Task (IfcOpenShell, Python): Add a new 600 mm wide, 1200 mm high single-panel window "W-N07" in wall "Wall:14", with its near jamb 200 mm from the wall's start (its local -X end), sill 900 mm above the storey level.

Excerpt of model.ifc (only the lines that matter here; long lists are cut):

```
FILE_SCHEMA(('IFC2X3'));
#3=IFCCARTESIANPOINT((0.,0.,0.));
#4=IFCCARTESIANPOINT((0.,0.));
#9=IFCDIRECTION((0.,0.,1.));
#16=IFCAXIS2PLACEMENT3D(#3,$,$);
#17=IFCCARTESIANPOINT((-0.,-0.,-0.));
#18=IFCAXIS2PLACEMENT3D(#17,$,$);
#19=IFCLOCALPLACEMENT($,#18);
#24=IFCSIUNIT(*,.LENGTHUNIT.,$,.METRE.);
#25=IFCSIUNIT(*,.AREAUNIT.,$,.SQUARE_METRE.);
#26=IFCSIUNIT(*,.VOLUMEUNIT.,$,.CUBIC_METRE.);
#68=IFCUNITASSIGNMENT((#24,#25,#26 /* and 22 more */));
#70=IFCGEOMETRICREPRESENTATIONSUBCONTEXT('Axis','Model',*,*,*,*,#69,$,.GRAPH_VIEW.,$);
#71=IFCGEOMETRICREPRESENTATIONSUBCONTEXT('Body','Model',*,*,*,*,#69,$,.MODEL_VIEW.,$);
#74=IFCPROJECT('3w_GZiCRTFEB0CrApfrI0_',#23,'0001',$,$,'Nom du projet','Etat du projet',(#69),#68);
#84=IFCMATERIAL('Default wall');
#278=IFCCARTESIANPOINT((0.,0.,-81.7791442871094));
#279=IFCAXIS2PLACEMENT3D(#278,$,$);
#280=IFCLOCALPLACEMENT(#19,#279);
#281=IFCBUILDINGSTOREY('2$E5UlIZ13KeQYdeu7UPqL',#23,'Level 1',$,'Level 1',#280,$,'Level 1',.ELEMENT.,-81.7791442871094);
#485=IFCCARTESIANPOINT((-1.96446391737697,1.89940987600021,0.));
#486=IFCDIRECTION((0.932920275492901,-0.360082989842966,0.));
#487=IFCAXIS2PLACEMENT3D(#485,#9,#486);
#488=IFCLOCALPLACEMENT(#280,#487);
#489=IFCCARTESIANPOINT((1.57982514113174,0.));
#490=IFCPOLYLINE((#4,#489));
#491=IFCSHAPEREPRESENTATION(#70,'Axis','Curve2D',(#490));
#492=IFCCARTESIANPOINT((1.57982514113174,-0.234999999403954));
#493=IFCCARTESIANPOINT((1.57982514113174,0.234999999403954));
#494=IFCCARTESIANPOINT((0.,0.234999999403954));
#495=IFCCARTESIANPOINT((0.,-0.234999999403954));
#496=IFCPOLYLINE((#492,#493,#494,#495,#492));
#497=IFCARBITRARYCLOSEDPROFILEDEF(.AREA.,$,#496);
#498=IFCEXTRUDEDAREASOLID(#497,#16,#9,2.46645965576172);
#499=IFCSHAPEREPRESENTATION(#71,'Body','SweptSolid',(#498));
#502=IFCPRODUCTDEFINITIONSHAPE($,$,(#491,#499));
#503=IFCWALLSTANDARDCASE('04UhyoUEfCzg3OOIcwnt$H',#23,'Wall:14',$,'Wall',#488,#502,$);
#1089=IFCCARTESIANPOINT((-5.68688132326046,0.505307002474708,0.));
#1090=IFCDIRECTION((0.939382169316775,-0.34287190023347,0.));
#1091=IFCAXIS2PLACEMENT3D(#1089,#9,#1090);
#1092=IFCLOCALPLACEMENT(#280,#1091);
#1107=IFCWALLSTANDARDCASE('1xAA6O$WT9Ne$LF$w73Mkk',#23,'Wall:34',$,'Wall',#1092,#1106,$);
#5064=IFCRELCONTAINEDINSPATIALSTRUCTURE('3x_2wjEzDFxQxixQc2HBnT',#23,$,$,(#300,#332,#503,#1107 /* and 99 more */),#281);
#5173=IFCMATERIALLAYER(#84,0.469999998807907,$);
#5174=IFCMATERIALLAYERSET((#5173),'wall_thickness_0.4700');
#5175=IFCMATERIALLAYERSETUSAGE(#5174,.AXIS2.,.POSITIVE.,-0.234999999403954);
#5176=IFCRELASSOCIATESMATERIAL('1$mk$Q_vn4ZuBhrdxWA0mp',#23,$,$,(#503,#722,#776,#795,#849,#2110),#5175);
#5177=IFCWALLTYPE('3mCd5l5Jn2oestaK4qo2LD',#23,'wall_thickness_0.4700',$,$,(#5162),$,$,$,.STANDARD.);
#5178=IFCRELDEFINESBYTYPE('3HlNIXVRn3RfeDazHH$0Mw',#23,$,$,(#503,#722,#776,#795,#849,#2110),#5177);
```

```python
import numpy as np
import ifcopenshell
import ifcopenshell.api.feature
import ifcopenshell.api.geometry
import ifcopenshell.api.root
import ifcopenshell.api.spatial
import ifcopenshell.api.type
import ifcopenshell.geom
import ifcopenshell.util.element
import ifcopenshell.util.placement
import ifcopenshell.util.representation
import ifcopenshell.util.shape
import ifcopenshell.util.unit

model = ifcopenshell.open("model.ifc")
unit_scale = ifcopenshell.util.unit.calculate_unit_scale(model)
settings = ifcopenshell.geom.settings()


def volume(element):
    """Net volume in cubic metres, openings subtracted."""
    shape = ifcopenshell.geom.create_shape(settings, element)
    return ifcopenshell.util.shape.get_volume(shape.geometry)


wall = model.by_id(503)
storey = ifcopenshell.util.element.get_container(wall, ifc_class="IfcBuildingStorey")
context = ifcopenshell.util.representation.get_context(model, "Model", "Body", "MODEL_VIEW")
before = volume(wall)

width, height, from_end, sill = 0.6, 1.2, 0.2, 0.9  # metres

# The wall runs along its own X axis, and the end named is its -X end.
wall_shape = ifcopenshell.geom.create_shape(settings, wall)
x, y, z = ifcopenshell.util.shape.get_vertices(wall_shape.geometry).T
start = x.min() + from_end
face, thickness = float(y.min()), float(y.max() - y.min())
wall_matrix = ifcopenshell.util.placement.get_local_placement(wall.ObjectPlacement)
level = ifcopenshell.util.placement.get_local_placement(storey.ObjectPlacement)[2, 3]


def in_wall(x, y):
    """Placement at x, y metres in the wall's axes, at sill height."""
    matrix = wall_matrix.copy()
    matrix[:, 3] = wall_matrix @ np.array([x / unit_scale, y / unit_scale, 0.0, 1.0])
    matrix[2, 3] = level + sill / unit_scale
    return matrix


# Opening: a box that overshoots both wall faces by 50 mm.
opening = ifcopenshell.api.root.create_entity(model, ifc_class="IfcOpeningElement")
box = ifcopenshell.api.geometry.add_wall_representation(
    model, context=context, length=width, height=height, thickness=thickness + 0.1
)
ifcopenshell.api.geometry.assign_representation(model, product=opening, representation=box)
ifcopenshell.api.geometry.edit_object_placement(model, product=opening, matrix=in_wall(start, face - 0.05), is_si=False)
ifcopenshell.api.feature.add_feature(model, feature=opening, element=wall)

window = ifcopenshell.api.root.create_entity(model, ifc_class="IfcWindow", name="W-N07")
window.OverallWidth, window.OverallHeight = width / unit_scale, height / unit_scale
body = ifcopenshell.api.geometry.add_window_representation(
    model,
    context=context,
    overall_width=window.OverallWidth,
    overall_height=window.OverallHeight,
    partition_type="SINGLE_PANEL",
)
ifcopenshell.api.geometry.assign_representation(model, product=window, representation=body)
ifcopenshell.api.spatial.assign_container(model, products=[window], relating_structure=storey)
fills = ifcopenshell.api.feature.add_filling(model, opening=opening, element=window)
fills.OwnerHistory = window.OwnerHistory  # required in IFC2X3

# IFC2X3 keeps the operation on the window style.
style = ifcopenshell.api.root.create_entity(model, ifc_class="IfcWindowStyle", name="W-N07")
style.OperationType, style.ConstructionType = "SINGLE_PANEL", "NOTDEFINED"
style.ParameterTakesPrecedence = style.Sizeable = False
ifcopenshell.api.type.assign_type(model, related_objects=[window], relating_type=style)

# Centre the window in the wall's thickness.
ifcopenshell.api.geometry.edit_object_placement(model, product=window, matrix=in_wall(start, face), is_si=False)
window_shape = ifcopenshell.geom.create_shape(settings, window)
depth = ifcopenshell.util.shape.get_vertices(window_shape.geometry)[:, 1]
offset = face + thickness / 2 - (depth.min() + depth.max()) / 2
ifcopenshell.api.geometry.edit_object_placement(model, product=window, matrix=in_wall(start, offset), is_si=False)

after = volume(wall)

print(f"wall volume {before:.3f} -> {after:.3f} m3")

model.write("model_edited.ifc")
```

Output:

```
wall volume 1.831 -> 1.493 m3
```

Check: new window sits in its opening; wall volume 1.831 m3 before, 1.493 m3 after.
